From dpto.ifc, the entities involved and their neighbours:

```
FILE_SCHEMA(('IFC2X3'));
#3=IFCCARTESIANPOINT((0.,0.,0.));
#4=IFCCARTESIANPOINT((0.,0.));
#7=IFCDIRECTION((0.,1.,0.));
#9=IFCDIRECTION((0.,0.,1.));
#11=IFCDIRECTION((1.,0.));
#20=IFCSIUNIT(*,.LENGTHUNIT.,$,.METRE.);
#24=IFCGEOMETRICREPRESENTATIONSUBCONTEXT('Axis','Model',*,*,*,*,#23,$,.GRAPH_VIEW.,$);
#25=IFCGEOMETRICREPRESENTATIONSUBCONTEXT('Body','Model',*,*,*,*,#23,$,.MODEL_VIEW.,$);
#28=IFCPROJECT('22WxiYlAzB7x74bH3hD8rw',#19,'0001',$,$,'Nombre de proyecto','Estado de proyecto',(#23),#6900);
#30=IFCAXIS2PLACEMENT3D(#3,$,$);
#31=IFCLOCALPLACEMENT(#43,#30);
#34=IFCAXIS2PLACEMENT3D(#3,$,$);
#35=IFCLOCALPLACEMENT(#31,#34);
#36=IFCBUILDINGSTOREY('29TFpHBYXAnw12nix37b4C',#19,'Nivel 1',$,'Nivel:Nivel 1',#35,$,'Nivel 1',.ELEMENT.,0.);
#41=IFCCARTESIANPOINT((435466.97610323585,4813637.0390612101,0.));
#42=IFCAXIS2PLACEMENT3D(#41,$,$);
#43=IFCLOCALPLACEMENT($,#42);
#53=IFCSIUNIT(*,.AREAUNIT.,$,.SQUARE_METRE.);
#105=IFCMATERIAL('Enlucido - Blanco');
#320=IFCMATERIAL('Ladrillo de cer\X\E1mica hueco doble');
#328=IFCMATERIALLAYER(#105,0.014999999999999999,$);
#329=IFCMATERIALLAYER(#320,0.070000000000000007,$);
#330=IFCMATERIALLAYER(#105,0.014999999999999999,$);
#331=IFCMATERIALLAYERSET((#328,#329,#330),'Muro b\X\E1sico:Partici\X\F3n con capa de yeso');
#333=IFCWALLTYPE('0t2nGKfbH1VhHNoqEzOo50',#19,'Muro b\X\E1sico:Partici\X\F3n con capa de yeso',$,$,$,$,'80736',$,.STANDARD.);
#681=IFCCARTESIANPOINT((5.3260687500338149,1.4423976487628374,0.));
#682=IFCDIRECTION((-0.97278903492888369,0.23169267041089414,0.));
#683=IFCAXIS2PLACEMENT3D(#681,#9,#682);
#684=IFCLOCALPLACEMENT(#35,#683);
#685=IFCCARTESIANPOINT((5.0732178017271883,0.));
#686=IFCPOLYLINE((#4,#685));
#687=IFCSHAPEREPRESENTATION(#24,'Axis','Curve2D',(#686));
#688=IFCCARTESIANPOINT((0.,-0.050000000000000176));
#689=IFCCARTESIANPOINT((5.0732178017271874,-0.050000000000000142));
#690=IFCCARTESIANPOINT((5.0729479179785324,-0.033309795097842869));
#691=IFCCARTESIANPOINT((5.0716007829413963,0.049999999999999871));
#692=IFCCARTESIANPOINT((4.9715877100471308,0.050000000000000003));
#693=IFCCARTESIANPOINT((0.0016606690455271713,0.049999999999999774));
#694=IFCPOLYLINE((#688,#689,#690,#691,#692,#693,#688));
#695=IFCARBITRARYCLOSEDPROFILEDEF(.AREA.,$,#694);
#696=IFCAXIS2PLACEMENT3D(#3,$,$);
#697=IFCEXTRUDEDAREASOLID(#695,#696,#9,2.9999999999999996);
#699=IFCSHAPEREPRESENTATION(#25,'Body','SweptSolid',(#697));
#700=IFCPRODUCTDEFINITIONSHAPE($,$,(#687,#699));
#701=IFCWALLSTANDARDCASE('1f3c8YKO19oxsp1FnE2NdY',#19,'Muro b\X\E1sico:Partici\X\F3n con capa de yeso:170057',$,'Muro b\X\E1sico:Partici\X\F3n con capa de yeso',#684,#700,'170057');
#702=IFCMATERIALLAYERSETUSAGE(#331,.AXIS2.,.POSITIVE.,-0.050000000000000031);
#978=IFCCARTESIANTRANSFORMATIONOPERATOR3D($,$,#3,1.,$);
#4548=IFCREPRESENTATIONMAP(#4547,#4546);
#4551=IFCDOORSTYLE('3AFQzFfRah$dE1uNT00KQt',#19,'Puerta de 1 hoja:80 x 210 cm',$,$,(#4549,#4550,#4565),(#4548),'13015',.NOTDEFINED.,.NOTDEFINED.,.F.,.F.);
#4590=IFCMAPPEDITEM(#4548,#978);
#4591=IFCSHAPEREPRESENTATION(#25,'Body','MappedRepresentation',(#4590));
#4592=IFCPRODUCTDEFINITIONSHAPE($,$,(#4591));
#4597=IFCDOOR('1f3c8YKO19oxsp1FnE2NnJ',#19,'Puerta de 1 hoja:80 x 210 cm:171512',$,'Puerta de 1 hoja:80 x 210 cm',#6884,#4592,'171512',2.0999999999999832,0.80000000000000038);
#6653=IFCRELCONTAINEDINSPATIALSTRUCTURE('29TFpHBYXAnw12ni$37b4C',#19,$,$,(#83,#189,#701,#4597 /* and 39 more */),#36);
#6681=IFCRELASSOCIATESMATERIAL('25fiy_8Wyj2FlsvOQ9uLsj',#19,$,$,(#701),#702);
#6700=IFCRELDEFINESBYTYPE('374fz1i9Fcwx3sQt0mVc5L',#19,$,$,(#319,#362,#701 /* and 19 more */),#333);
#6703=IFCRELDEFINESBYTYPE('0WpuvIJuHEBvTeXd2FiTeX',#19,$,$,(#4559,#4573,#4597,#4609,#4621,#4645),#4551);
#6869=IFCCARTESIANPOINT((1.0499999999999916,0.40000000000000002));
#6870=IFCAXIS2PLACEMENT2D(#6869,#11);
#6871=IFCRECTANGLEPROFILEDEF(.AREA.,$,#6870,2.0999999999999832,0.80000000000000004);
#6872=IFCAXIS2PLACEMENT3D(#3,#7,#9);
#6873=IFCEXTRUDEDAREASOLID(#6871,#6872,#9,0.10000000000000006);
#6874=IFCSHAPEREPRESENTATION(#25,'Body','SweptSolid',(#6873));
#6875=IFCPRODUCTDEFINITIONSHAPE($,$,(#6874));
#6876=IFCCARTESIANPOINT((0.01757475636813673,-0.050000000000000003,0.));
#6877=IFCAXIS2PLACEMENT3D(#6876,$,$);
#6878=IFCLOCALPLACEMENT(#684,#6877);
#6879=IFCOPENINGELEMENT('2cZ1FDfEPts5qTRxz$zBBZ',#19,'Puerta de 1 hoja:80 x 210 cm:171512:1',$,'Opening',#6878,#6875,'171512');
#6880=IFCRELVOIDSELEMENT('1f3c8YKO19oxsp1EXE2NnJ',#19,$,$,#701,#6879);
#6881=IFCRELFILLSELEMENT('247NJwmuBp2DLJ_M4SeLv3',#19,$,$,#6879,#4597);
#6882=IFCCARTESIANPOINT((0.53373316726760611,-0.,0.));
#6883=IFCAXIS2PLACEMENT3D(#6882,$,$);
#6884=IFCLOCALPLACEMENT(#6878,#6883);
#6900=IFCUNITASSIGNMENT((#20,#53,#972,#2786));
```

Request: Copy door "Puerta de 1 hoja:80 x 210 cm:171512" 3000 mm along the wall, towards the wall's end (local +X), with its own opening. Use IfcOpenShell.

```python
import ifcopenshell
import ifcopenshell.api.feature
import ifcopenshell.api.geometry
import ifcopenshell.api.root
import ifcopenshell.geom
import ifcopenshell.util.element
import ifcopenshell.util.placement
import ifcopenshell.util.shape
import ifcopenshell.util.unit

model = ifcopenshell.open("dpto.ifc")
unit_scale = ifcopenshell.util.unit.calculate_unit_scale(model)
settings = ifcopenshell.geom.settings()


def volume(element):
    """Net volume in cubic metres, openings subtracted."""
    shape = ifcopenshell.geom.create_shape(settings, element)
    return ifcopenshell.util.shape.get_volume(shape.geometry)


def reuse_history(source, copy):
    """copy_class also copies each property set's owner history, people and application; keep the originals."""
    for rel in copy.IsDefinedBy:
        if rel.is_a("IfcRelDefinesByProperties") and (history := rel.RelatingPropertyDefinition.OwnerHistory):
            rel.RelatingPropertyDefinition.OwnerHistory = source.OwnerHistory
            ifcopenshell.util.element.remove_deep2(model, history)


door = model.by_guid("1f3c8YKO19oxsp1FnE2NnJ")
opening = door.FillsVoids[0].RelatingOpeningElement
wall = opening.VoidsElements[0].RelatingBuildingElement
before = volume(wall)
shift = ifcopenshell.util.placement.get_local_placement(wall.ObjectPlacement)[:3, 0] * 3 / unit_scale

# copy_class copies the void relationship, type, container and properties, but no geometry.
new_opening = ifcopenshell.api.root.copy_class(model, product=opening)
new_opening.Representation = ifcopenshell.util.element.copy_deep(
    model, opening.Representation, exclude=["IfcGeometricRepresentationContext", "IfcRepresentationMap"]
)
new_opening.Name = "Puerta de 1 hoja:80 x 210 cm"
new_opening.Tag = None
new_door = ifcopenshell.api.root.copy_class(model, product=door)
new_door.Representation = ifcopenshell.util.element.copy_deep(
    model, door.Representation, exclude=["IfcGeometricRepresentationContext", "IfcRepresentationMap"]
)
new_door.Name = "Puerta de 1 hoja:80 x 210 cm"
new_door.Tag = None
reuse_history(door, new_door)
fills = ifcopenshell.api.feature.add_filling(model, opening=new_opening, element=new_door)
fills.OwnerHistory = new_door.OwnerHistory  # required in IFC2X3

for old, new in ((opening, new_opening), (door, new_door)):
    matrix = ifcopenshell.util.placement.get_local_placement(old.ObjectPlacement)
    matrix[:3, 3] += shift
    ifcopenshell.api.geometry.edit_object_placement(model, product=new, matrix=matrix, is_si=False)

after = volume(wall)

print(f"wall volume {before:.3f} -> {after:.3f} m3")

model.write("dpto_updated.ifc")
```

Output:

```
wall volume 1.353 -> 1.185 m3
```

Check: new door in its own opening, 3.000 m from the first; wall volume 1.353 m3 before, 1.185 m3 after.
